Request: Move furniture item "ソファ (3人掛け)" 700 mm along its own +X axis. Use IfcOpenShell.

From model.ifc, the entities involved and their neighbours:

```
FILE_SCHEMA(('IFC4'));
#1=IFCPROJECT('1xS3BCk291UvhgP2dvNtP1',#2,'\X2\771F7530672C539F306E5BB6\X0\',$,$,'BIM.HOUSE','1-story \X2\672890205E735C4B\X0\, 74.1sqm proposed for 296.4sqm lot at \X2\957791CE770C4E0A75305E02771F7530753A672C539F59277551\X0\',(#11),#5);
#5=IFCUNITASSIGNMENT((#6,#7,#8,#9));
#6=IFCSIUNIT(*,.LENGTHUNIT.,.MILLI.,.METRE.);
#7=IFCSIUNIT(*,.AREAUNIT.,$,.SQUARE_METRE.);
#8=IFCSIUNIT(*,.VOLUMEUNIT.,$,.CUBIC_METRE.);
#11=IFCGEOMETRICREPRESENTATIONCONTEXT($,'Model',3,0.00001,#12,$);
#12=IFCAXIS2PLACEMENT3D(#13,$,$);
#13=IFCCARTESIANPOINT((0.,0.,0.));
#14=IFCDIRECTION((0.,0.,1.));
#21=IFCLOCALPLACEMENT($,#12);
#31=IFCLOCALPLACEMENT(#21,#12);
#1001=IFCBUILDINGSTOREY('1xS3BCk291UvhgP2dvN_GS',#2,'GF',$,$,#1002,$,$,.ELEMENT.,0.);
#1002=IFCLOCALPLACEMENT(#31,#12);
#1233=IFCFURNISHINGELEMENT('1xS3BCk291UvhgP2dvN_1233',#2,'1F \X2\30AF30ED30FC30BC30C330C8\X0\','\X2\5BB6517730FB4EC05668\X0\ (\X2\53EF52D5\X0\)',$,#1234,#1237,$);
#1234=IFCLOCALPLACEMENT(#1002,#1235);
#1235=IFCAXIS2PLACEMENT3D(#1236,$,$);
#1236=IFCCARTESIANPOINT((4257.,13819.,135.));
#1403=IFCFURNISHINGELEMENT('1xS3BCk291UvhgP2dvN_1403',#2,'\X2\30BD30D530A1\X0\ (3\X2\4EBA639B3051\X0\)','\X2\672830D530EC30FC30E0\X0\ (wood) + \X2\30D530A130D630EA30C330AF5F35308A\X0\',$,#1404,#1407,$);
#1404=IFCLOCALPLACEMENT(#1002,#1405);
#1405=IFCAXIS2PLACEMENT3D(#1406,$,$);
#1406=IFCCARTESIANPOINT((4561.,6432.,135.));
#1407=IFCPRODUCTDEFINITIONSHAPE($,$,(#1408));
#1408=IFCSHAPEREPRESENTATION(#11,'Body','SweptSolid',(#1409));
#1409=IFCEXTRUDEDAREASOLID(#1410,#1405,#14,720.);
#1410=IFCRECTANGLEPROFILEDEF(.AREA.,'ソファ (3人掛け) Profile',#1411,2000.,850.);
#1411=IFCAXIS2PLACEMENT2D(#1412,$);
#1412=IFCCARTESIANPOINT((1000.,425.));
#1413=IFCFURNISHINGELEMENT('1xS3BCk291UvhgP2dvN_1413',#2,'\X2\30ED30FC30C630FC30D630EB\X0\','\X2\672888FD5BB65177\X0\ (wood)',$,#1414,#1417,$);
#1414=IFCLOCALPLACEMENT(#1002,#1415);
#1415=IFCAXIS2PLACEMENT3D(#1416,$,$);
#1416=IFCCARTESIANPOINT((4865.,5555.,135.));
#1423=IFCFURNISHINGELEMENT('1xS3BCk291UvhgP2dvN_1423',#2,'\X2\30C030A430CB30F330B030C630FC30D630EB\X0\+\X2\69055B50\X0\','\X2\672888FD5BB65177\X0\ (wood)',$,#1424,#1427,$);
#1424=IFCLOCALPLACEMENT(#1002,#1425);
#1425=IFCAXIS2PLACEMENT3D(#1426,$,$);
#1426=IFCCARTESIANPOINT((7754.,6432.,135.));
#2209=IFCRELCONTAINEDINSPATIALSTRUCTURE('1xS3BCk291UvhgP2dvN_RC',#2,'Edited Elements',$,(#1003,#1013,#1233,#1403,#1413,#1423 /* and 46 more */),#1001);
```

```python
import ifcopenshell
import ifcopenshell.api.geometry
import ifcopenshell.util.placement

model = ifcopenshell.open("model.ifc")

item = model.by_guid("1xS3BCk291UvhgP2dvN_1403")
matrix = ifcopenshell.util.placement.get_local_placement(item.ObjectPlacement)
matrix[:3, 3] += matrix[:3, 0] * 700.0
ifcopenshell.api.geometry.edit_object_placement(model, product=item, matrix=matrix, is_si=False)

print(ifcopenshell.util.placement.get_local_placement(item.ObjectPlacement).round(3) + 0.0)

model.write("model_edited.ifc")
```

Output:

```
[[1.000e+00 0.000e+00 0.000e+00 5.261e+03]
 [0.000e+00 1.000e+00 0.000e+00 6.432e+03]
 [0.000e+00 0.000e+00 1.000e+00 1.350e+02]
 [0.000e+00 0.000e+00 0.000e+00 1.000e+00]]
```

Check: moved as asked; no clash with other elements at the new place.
